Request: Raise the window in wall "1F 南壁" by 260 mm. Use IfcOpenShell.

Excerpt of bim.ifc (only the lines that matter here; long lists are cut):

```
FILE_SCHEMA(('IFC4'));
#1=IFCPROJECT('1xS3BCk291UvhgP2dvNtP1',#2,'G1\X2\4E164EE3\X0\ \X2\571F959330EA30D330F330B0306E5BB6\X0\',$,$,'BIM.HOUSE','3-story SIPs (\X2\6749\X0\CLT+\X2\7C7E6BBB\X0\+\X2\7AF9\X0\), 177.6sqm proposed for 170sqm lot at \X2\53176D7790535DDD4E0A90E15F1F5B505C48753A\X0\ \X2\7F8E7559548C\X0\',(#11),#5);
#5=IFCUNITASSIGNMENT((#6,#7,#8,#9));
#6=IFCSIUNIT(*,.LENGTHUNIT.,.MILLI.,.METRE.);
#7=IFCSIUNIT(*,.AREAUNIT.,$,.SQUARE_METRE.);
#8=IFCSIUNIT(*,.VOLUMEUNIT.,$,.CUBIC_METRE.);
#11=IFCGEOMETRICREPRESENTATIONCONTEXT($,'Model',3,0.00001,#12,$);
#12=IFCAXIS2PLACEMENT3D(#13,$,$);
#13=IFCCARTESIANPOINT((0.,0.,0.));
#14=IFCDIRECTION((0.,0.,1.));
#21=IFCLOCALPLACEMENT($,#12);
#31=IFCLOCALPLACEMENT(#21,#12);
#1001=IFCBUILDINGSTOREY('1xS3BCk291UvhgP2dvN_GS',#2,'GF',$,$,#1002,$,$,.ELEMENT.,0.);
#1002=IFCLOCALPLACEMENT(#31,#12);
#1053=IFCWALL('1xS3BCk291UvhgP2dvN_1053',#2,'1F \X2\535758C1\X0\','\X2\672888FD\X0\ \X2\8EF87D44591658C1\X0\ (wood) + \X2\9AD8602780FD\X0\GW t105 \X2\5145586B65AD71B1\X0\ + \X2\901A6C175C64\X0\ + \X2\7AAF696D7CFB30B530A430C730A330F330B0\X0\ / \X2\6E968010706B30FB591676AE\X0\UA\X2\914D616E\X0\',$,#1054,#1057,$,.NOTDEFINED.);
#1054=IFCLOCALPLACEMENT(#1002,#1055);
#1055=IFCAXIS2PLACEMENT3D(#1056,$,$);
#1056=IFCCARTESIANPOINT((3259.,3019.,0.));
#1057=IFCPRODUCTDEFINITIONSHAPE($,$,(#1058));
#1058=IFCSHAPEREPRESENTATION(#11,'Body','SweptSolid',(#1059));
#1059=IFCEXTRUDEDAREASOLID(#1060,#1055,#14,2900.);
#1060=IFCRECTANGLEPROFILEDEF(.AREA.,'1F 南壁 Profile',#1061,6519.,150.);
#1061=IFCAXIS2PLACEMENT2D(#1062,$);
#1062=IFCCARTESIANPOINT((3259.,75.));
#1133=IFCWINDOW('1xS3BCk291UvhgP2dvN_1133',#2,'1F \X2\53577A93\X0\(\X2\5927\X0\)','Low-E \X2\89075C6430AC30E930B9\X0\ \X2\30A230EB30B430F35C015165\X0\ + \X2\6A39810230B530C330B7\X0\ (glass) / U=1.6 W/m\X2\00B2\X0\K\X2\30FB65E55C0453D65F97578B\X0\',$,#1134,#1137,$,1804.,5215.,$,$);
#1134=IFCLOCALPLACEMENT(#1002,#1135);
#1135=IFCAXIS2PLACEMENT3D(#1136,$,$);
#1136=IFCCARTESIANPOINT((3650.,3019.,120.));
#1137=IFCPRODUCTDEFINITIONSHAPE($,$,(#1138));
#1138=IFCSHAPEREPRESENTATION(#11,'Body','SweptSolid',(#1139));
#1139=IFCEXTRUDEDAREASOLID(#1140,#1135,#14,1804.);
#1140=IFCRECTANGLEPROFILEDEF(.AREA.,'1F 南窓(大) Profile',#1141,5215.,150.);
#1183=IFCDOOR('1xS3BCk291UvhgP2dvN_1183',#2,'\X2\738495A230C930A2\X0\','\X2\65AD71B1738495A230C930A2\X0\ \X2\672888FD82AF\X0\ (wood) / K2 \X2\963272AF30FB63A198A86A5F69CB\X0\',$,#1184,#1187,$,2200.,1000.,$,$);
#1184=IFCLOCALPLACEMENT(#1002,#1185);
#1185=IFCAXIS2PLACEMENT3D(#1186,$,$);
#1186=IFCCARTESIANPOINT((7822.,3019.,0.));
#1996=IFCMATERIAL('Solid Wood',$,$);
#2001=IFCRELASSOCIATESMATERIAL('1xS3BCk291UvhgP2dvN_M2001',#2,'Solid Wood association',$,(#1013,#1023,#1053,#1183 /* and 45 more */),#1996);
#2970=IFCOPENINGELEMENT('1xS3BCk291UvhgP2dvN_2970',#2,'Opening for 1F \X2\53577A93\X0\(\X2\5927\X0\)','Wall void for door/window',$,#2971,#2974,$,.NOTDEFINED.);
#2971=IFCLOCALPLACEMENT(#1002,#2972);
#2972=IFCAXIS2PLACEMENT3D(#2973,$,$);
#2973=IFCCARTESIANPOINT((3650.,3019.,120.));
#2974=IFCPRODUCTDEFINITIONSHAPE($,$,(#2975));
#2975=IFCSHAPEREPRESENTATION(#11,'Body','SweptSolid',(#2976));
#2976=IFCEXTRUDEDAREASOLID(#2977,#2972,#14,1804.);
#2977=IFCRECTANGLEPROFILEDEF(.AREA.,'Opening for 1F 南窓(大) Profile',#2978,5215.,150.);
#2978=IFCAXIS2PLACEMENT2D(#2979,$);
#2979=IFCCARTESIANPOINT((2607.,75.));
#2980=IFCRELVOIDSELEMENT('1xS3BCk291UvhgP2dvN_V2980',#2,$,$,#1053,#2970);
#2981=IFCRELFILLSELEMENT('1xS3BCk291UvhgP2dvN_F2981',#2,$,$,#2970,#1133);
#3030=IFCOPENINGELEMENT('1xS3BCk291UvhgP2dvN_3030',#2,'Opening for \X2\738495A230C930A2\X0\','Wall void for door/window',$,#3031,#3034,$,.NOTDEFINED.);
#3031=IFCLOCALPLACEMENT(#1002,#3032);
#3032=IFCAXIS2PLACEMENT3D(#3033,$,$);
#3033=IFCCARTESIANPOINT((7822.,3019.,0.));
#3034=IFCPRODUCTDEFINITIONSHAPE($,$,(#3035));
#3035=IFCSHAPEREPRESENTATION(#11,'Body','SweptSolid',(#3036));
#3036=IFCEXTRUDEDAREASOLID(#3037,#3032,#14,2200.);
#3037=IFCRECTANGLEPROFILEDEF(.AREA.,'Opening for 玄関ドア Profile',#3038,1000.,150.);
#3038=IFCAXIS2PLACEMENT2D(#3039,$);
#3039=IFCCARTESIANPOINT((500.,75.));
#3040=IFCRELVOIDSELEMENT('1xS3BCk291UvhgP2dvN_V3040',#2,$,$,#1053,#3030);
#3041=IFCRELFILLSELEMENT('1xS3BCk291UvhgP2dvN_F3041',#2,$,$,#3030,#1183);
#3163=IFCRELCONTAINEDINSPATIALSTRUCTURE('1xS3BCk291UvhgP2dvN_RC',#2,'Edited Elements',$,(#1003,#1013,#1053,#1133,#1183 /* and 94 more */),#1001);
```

```python
import numpy as np
import ifcopenshell
import ifcopenshell.api.geometry
import ifcopenshell.util.placement
import ifcopenshell.util.unit

model = ifcopenshell.open("bim.ifc")
unit_scale = ifcopenshell.util.unit.calculate_unit_scale(model)

window = model.by_guid("1xS3BCk291UvhgP2dvN_1133")
opening = window.FillsVoids[0].RelatingOpeningElement
dz = 260.0

shift = np.array([0.0, 0.0, dz])
# The window is not placed relative to its opening, so move both.
for product in (opening, window):
    matrix = ifcopenshell.util.placement.get_local_placement(product.ObjectPlacement)
    matrix[:3, 3] += shift
    ifcopenshell.api.geometry.edit_object_placement(model, product=product, matrix=matrix, is_si=False)

print(f"moved by {dz * unit_scale:+.3f} m")

model.write("bim-out.ifc")
```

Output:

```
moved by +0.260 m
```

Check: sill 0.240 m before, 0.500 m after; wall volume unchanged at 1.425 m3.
